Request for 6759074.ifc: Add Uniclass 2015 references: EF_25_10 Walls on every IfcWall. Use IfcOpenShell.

First a look at what the model holds.

```python
import ifcopenshell

model = ifcopenshell.open("6759074.ifc")
print(model.schema)
print("classifications:", [c.Name for c in model.by_type("IfcClassification")])
for ifc_class in ("IfcDoor", "IfcRoof", "IfcStair", "IfcWall", "IfcWindow"):
    print(ifc_class, len(model.by_type(ifc_class)))
```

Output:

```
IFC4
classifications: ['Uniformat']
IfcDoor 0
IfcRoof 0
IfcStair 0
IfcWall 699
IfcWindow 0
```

```python
import ifcopenshell
import ifcopenshell.api.classification

model = ifcopenshell.open("6759074.ifc")

system = ifcopenshell.api.classification.add_classification(model, classification="Uniclass 2015")

codes = {
    "IfcWall": ("EF_25_10", "Walls"),
}
for ifc_class, (code, name) in codes.items():
    products = model.by_type(ifc_class)
    ifcopenshell.api.classification.add_reference(
        model, products=products, classification=system, identification=code, name=name
    )
    print(code, len(products))

model.write("6759074_updated.ifc")
```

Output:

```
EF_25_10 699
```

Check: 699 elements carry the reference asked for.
